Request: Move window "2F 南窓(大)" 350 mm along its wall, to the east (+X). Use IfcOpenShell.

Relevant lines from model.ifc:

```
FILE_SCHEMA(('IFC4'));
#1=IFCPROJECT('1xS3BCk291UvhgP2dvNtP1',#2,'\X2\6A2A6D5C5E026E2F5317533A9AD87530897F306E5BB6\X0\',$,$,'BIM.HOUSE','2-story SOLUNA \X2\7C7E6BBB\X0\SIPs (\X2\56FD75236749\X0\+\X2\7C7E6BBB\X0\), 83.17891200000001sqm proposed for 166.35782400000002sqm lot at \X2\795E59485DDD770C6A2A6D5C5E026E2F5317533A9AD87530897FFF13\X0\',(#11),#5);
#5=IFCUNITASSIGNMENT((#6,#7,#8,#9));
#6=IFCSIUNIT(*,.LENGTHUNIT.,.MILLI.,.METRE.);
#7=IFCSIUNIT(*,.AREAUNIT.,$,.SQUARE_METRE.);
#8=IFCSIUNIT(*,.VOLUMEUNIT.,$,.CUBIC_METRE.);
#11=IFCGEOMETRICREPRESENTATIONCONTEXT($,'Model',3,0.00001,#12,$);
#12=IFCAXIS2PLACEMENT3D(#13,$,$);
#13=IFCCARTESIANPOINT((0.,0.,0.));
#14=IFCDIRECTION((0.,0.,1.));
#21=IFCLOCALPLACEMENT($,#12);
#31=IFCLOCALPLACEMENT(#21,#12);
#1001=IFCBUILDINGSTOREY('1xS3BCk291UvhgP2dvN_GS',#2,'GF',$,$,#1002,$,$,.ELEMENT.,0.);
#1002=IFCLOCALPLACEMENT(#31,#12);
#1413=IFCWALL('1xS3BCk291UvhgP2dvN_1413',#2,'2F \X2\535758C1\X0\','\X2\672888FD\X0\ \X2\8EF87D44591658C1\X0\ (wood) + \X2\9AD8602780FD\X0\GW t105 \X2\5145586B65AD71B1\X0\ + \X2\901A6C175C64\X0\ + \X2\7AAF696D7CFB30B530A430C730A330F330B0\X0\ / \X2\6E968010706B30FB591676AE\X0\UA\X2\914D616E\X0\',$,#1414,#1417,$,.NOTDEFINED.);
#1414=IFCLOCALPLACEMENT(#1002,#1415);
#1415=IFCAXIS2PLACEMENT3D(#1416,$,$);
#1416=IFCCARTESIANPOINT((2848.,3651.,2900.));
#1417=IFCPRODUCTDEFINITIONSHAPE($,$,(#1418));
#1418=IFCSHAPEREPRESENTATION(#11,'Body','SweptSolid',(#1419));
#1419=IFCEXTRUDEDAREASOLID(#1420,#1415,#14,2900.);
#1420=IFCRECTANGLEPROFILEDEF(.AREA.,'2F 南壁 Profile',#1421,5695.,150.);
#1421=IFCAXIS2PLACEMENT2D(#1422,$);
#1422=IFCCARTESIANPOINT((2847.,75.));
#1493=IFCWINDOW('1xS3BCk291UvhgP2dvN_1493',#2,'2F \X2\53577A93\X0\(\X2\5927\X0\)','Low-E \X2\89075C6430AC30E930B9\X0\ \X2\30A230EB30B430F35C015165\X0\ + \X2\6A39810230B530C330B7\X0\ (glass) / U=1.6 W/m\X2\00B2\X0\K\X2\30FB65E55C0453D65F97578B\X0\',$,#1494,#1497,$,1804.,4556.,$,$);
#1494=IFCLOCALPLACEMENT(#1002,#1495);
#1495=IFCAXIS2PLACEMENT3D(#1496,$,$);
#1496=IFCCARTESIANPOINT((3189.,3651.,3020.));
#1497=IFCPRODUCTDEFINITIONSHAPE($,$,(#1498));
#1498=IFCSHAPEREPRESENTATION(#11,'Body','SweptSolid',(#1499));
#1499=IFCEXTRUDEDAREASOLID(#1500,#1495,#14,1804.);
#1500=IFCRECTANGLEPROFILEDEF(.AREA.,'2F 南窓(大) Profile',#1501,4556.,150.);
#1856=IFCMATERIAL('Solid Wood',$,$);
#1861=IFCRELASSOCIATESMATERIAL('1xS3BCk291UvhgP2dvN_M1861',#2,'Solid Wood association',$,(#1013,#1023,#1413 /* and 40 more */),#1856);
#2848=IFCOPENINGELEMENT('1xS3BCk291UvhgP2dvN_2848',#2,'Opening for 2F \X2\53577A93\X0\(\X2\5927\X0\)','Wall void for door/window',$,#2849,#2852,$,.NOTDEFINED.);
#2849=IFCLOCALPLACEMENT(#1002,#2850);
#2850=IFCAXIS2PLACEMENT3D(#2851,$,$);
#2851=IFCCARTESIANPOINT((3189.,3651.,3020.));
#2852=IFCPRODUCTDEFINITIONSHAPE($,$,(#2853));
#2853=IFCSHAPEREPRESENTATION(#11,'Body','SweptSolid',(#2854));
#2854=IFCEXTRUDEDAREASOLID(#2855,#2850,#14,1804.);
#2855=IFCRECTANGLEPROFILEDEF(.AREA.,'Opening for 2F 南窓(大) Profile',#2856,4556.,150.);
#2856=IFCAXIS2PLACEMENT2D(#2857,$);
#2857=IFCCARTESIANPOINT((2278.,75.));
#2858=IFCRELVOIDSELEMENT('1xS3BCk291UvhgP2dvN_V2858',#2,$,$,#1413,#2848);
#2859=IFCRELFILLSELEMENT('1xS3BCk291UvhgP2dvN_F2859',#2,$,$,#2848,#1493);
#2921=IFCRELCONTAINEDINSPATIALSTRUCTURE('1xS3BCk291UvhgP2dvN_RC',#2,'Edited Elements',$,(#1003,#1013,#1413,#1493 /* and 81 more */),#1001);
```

```python
import ifcopenshell
import ifcopenshell.api.geometry
import ifcopenshell.util.placement
import ifcopenshell.util.unit

model = ifcopenshell.open("model.ifc")
unit_scale = ifcopenshell.util.unit.calculate_unit_scale(model)

window = model.by_id(1493)
opening = window.FillsVoids[0].RelatingOpeningElement
wall = opening.VoidsElements[0].RelatingBuildingElement

wall_matrix = ifcopenshell.util.placement.get_local_placement(wall.ObjectPlacement)
shift = wall_matrix[:3, 0] * 0.35 / unit_scale
before = ifcopenshell.util.placement.get_local_placement(window.ObjectPlacement)[:3, 3].copy()

# The window is not placed relative to its opening, so move both.
for product in (opening, window):
    matrix = ifcopenshell.util.placement.get_local_placement(product.ObjectPlacement)
    matrix[:3, 3] += shift
    ifcopenshell.api.geometry.edit_object_placement(model, product=product, matrix=matrix, is_si=False)

after = ifcopenshell.util.placement.get_local_placement(window.ObjectPlacement)[:3, 3]
print("window moved by", (after - before).round(3) + 0.0)

model.write("model_edited.ifc")
```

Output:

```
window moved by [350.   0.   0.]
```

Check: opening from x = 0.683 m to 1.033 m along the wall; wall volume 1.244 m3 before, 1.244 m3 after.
